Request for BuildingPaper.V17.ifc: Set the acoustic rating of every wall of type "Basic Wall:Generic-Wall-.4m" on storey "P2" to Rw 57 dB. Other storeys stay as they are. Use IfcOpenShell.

First a look at what the model holds.

```python
import ifcopenshell
import ifcopenshell.util.element

model = ifcopenshell.open("BuildingPaper.V17.ifc")
print(model.schema)
storey = next(s for s in model.by_type("IfcBuildingStorey") if s.Name == "P2")
walls = [e for e in ifcopenshell.util.element.get_decomposition(storey) if e.is_a("IfcWall")]
seen = {}
for e in walls:
    element_type = ifcopenshell.util.element.get_type(e)
    key = (element_type.Name if element_type != e and element_type else None, ifcopenshell.util.element.get_pset(e, "Pset_WallCommon", "AcousticRating"))
    seen[key] = seen.get(key, 0) + 1
for (name, value), count in sorted(seen.items(), key=str):
    print(count, "x", name, "|", value)
```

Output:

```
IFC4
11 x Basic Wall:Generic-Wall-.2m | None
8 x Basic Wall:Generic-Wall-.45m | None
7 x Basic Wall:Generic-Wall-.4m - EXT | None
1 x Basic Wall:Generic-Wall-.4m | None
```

```python
import ifcopenshell
import ifcopenshell.api.pset
import ifcopenshell.util.element

model = ifcopenshell.open("BuildingPaper.V17.ifc")

storey = next(s for s in model.by_type("IfcBuildingStorey") if s.Name == "P2")
walls = [e for e in ifcopenshell.util.element.get_decomposition(storey) if e.is_a("IfcWall")]

count = 0
for e in walls:
    element_type = ifcopenshell.util.element.get_type(e)
    if element_type in (None, e) or element_type.Name != "Basic Wall:Generic-Wall-.4m":
        continue
    # add_pset returns the element's existing set when there is one.
    pset = ifcopenshell.api.pset.add_pset(model, product=e, name="Pset_WallCommon")
    ifcopenshell.api.pset.edit_pset(model, pset=pset, properties={"AcousticRating": "Rw 57 dB"})
    count += 1

print(count, "walls updated")

model.write("BuildingPaper.V17_edited.ifc")
```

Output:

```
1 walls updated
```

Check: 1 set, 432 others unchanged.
